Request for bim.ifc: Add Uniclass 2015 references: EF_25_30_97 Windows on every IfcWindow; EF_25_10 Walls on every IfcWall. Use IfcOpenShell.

First a look at what the model holds.

```python
import ifcopenshell

model = ifcopenshell.open("bim.ifc")
print(model.schema)
print("classifications:", [c.Name for c in model.by_type("IfcClassification")])
for ifc_class in ("IfcDoor", "IfcRoof", "IfcStair", "IfcWall", "IfcWindow"):
    print(ifc_class, len(model.by_type(ifc_class)))
```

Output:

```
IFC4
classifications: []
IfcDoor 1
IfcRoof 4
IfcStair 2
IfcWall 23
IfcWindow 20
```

```python
import ifcopenshell
import ifcopenshell.api.classification

model = ifcopenshell.open("bim.ifc")

system = ifcopenshell.api.classification.add_classification(model, classification="Uniclass 2015")

codes = {
    "IfcWindow": ("EF_25_30_97", "Windows"),
    "IfcWall": ("EF_25_10", "Walls"),
}
for ifc_class, (code, name) in codes.items():
    products = model.by_type(ifc_class)
    ifcopenshell.api.classification.add_reference(
        model, products=products, classification=system, identification=code, name=name
    )
    print(code, len(products))

model.write("bim-out.ifc")
```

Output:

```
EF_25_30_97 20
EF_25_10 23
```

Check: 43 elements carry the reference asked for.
